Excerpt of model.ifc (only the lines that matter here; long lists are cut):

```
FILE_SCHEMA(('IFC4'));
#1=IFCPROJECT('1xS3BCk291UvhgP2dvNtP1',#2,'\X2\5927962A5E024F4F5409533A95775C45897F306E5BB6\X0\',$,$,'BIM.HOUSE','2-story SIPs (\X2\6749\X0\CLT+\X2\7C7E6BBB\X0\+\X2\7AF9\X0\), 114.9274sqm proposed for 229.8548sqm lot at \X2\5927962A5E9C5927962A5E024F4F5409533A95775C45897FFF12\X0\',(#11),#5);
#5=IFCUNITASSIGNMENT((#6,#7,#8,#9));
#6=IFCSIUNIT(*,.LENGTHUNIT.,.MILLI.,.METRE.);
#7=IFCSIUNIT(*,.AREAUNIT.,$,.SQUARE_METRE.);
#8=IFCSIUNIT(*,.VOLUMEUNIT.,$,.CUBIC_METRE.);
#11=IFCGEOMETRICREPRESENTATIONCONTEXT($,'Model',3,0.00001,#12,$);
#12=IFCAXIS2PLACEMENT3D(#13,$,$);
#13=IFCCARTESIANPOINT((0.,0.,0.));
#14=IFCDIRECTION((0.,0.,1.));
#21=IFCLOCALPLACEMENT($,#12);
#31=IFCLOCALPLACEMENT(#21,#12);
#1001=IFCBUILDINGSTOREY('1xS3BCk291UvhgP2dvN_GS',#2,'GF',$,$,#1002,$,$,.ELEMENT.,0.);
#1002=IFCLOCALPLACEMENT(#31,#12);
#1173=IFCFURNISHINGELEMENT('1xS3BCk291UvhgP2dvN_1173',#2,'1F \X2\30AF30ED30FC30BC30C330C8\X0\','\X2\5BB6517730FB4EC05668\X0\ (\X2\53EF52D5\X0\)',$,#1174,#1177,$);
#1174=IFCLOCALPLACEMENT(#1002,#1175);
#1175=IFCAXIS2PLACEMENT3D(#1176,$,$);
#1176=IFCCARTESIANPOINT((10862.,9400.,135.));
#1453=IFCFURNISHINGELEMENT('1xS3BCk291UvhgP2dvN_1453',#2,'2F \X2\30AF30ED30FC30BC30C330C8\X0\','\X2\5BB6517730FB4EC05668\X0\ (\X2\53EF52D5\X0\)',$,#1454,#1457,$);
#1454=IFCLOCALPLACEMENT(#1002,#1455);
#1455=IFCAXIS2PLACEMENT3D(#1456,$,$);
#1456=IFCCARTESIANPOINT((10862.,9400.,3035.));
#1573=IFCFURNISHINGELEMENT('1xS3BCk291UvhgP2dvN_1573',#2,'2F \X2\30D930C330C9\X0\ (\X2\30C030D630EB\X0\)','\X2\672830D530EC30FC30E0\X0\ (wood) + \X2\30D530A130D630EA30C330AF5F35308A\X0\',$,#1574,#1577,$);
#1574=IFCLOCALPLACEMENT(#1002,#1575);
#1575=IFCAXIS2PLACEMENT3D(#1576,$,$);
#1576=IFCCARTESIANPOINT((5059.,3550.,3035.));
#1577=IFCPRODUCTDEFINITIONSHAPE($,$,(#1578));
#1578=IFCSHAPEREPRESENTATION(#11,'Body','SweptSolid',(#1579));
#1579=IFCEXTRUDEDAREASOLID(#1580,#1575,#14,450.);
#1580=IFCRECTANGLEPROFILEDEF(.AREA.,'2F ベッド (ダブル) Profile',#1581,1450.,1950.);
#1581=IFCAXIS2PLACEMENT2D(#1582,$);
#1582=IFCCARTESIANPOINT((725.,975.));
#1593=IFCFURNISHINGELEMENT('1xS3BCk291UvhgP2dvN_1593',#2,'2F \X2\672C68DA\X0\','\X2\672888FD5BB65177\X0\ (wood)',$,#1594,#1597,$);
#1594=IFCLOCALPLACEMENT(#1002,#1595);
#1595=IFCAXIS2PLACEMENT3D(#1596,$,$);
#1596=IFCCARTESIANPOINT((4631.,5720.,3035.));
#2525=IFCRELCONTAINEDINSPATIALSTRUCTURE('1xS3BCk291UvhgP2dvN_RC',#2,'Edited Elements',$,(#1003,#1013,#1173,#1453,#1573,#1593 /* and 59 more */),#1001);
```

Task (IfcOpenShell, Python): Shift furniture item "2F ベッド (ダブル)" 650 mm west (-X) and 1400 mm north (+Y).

```python
import ifcopenshell
import ifcopenshell.api.geometry
import ifcopenshell.util.placement

model = ifcopenshell.open("model.ifc")

item = model.by_guid("1xS3BCk291UvhgP2dvN_1573")
matrix = ifcopenshell.util.placement.get_local_placement(item.ObjectPlacement)
matrix[0, 3] -= 650.0
matrix[1, 3] += 1400.0
ifcopenshell.api.geometry.edit_object_placement(model, product=item, matrix=matrix, is_si=False)

print(ifcopenshell.util.placement.get_local_placement(item.ObjectPlacement).round(3) + 0.0)

model.write("model_rev.ifc")
```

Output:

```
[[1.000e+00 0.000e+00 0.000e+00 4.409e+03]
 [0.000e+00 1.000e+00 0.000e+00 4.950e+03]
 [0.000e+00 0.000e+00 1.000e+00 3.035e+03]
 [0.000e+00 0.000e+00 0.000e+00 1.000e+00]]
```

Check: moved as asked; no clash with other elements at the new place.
